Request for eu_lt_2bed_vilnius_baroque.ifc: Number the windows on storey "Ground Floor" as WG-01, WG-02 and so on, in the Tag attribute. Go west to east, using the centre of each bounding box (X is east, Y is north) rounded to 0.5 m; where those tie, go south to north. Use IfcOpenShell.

First a look at what the model holds.

```python
import ifcopenshell
import ifcopenshell.util.element
import ifcopenshell.util.placement

model = ifcopenshell.open("eu_lt_2bed_vilnius_baroque.ifc")
print(model.schema)
storey = next(s for s in model.by_type("IfcBuildingStorey") if s.Name == "Ground Floor")
windows = [e for e in ifcopenshell.util.element.get_decomposition(storey) if e.is_a("IfcWindow")]
for e in sorted(windows, key=lambda e: e.id()):
    origin = ifcopenshell.util.placement.get_local_placement(e.ObjectPlacement)[:3, 3]
    print(e.id(), e.Tag, e.Name, origin.round(2) + 0.0, sep=" | ")
```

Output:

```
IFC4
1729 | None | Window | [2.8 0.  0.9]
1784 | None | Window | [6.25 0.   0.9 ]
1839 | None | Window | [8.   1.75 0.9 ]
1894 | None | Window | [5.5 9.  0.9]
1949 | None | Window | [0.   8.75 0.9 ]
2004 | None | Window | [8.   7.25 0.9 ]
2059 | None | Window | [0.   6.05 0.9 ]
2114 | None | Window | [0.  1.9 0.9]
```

```python
import ifcopenshell
import ifcopenshell.geom
import ifcopenshell.util.element
import ifcopenshell.util.shape

model = ifcopenshell.open("eu_lt_2bed_vilnius_baroque.ifc")
settings = ifcopenshell.geom.settings()
settings.set("use-world-coords", True)


def centre(element):
    shape = ifcopenshell.geom.create_shape(settings, element)
    return ifcopenshell.util.shape.get_bbox_centroid(shape.geometry)


storey = next(s for s in model.by_type("IfcBuildingStorey") if s.Name == "Ground Floor")
windows = [e for e in ifcopenshell.util.element.get_decomposition(storey) if e.is_a("IfcWindow")]

# Insertion points can sit at a corner or the storey origin, so sort by the geometry (in metres).
centres = {e: centre(e) for e in windows}
windows.sort(key=lambda e: (round(centres[e][0] / 0.5), centres[e][1]))

for i, e in enumerate(windows, start=1):
    number = f"WG-{i:02d}"
    e.Tag = number
    print(e.id(), number)

model.write("eu_lt_2bed_vilnius_baroque_updated.ifc")
```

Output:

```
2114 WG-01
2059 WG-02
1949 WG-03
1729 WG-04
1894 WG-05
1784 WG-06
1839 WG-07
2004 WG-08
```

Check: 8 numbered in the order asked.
